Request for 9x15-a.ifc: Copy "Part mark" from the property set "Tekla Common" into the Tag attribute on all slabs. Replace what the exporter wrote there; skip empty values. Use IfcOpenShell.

First a look at what the model holds.

```python
import ifcopenshell
import ifcopenshell.util.element

model = ifcopenshell.open("9x15-a.ifc")
print(model.schema)
slabs = model.by_type("IfcSlab")
print(len(slabs), "slabs")
for e in slabs[:8]:
    source = ifcopenshell.util.element.get_pset(e, "Tekla Common", "Part mark")
    target = e.Tag
    print(e.id(), repr(source), repr(target), sep=" | ")
```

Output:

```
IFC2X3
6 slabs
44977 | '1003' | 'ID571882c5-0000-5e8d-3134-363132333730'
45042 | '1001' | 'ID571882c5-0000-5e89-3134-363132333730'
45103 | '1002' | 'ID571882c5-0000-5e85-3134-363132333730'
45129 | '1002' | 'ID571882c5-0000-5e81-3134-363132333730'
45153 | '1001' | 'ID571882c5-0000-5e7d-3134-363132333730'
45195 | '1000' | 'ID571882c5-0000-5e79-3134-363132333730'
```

```python
import ifcopenshell
import ifcopenshell.util.element

model = ifcopenshell.open("9x15-a.ifc")

count = 0
for e in model.by_type("IfcSlab"):
    value = ifcopenshell.util.element.get_pset(e, "Tekla Common", "Part mark")
    current = e.Tag
    if not value or not value.strip() or current == value:
        continue
    e.Tag = value
    count += 1

print(count, "slabs updated")

model.write("9x15-a_rev.ifc")
```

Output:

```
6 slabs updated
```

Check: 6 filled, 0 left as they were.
